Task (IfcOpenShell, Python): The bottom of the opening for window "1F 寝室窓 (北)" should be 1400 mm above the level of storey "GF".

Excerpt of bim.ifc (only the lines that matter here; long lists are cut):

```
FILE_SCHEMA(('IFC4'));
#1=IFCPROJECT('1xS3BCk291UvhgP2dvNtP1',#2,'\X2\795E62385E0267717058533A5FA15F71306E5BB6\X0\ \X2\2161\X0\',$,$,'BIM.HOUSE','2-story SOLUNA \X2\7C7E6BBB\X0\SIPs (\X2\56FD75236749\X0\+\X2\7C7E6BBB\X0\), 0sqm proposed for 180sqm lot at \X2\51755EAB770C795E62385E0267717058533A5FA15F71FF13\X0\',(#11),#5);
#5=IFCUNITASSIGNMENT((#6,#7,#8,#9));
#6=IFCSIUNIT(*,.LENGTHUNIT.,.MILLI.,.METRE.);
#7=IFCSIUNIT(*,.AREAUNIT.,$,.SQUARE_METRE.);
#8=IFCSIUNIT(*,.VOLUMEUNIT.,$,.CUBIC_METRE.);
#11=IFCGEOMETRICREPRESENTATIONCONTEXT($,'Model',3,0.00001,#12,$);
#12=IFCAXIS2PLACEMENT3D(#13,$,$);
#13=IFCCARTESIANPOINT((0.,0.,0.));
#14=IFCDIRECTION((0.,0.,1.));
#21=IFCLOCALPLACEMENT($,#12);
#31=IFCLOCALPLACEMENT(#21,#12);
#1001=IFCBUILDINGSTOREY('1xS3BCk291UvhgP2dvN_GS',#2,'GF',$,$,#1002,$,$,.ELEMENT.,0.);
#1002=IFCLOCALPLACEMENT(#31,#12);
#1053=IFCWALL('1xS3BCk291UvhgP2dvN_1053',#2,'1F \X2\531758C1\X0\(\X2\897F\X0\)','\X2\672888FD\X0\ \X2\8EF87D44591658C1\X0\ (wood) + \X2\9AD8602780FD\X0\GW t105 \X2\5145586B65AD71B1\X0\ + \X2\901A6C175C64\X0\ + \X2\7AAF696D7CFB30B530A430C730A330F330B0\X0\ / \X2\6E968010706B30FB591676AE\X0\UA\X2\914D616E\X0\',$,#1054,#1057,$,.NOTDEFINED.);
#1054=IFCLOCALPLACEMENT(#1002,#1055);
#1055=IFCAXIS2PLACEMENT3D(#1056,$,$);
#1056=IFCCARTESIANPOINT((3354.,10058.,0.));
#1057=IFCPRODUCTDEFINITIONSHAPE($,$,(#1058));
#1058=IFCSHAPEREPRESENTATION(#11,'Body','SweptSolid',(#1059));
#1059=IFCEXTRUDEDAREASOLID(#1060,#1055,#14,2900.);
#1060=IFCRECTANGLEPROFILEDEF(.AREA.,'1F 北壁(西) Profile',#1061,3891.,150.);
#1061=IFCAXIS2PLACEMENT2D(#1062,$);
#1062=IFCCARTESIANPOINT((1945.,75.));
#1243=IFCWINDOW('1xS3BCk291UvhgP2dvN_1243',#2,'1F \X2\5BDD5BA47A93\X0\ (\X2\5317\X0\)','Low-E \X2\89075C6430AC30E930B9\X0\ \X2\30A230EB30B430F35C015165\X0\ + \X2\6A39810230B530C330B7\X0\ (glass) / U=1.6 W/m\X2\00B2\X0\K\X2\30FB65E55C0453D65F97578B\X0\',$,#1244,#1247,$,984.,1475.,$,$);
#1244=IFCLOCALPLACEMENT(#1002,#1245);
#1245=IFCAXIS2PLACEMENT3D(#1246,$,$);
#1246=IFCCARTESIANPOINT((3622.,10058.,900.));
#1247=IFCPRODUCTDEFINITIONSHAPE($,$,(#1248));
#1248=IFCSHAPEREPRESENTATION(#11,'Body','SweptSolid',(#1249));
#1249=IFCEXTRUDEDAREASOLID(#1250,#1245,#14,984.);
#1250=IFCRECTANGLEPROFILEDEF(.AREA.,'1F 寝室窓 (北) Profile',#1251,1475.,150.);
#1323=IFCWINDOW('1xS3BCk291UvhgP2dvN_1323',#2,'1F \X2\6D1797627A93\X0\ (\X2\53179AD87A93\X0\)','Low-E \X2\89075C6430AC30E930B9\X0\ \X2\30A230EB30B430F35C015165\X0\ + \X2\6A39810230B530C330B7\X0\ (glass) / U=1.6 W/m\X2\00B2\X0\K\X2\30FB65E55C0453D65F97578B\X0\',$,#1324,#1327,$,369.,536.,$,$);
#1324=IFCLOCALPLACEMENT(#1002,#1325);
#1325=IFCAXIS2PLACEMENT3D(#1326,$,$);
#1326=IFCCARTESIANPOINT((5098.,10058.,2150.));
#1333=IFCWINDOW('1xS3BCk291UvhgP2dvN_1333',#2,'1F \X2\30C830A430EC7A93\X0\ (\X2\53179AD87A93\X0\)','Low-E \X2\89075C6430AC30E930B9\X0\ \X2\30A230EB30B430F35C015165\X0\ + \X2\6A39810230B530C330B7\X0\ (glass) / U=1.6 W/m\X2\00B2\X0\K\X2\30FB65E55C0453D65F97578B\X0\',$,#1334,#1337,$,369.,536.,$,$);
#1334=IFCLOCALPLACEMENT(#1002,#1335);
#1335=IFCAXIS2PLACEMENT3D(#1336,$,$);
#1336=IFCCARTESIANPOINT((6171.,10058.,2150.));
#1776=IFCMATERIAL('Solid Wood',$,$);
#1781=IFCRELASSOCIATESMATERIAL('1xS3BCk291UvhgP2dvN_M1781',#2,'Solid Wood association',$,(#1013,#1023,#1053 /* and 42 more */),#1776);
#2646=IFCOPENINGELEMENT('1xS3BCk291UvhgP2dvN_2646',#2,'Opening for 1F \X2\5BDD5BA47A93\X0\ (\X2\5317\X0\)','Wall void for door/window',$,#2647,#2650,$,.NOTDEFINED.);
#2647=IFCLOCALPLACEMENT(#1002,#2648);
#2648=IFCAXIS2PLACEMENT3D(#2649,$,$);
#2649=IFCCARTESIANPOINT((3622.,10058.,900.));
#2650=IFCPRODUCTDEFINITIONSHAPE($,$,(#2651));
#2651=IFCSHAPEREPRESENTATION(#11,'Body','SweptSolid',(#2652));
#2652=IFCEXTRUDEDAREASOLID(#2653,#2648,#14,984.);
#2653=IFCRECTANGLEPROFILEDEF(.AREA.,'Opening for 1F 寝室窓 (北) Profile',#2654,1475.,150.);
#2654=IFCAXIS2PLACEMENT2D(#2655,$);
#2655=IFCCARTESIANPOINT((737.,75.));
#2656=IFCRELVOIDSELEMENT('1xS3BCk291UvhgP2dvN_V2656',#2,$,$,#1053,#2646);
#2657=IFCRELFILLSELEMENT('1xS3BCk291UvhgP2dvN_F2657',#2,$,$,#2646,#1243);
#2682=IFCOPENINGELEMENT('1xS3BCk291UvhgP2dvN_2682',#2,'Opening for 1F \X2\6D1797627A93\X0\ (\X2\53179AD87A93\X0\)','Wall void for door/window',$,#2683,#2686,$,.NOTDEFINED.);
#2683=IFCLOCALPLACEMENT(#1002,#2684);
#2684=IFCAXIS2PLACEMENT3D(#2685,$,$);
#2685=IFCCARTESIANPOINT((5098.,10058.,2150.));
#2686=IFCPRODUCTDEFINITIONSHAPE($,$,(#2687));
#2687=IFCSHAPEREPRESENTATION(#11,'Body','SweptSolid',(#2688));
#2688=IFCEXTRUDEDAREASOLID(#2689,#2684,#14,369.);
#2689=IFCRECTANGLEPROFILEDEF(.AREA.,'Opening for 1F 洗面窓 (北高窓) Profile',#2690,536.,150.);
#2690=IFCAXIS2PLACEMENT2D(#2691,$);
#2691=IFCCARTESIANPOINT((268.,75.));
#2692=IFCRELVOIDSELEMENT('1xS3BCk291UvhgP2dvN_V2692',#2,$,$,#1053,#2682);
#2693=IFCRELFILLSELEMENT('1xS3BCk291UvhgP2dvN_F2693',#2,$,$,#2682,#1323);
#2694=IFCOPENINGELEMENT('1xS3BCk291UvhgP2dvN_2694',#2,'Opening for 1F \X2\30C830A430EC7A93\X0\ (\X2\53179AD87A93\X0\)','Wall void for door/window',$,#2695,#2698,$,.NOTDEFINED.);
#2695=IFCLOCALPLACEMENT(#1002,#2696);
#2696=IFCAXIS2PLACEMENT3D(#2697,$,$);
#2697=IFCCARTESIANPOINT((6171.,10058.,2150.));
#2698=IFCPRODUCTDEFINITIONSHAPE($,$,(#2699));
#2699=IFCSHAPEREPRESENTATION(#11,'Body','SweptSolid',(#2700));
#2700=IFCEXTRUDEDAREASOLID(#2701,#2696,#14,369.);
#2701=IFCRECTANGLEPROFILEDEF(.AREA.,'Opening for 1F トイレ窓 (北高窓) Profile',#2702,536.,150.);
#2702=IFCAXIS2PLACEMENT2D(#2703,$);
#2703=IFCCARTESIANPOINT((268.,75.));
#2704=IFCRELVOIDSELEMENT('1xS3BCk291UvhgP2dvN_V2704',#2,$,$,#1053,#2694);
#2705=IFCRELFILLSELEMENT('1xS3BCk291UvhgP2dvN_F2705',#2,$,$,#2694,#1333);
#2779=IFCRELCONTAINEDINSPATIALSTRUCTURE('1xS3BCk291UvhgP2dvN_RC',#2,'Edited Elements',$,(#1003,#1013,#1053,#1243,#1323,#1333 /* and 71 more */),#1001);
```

```python
import numpy as np
import ifcopenshell
import ifcopenshell.api.geometry
import ifcopenshell.geom
import ifcopenshell.util.element
import ifcopenshell.util.placement
import ifcopenshell.util.shape
import ifcopenshell.util.unit

model = ifcopenshell.open("bim.ifc")
unit_scale = ifcopenshell.util.unit.calculate_unit_scale(model)

window = model.by_guid("1xS3BCk291UvhgP2dvN_1243")
opening = window.FillsVoids[0].RelatingOpeningElement
storey = ifcopenshell.util.element.get_container(window, ifc_class="IfcBuildingStorey")
level = ifcopenshell.util.placement.get_local_placement(storey.ObjectPlacement)[2, 3]

# The opening's origin need not be at the sill, so measure its lowest point.
shape = ifcopenshell.geom.create_shape(ifcopenshell.geom.settings(), opening)
bottom = ifcopenshell.util.shape.get_shape_bottom_elevation(shape, shape.geometry) / unit_scale
dz = level + 1400.0 - bottom

shift = np.array([0.0, 0.0, dz])
# The window is not placed relative to its opening, so move both.
for product in (opening, window):
    matrix = ifcopenshell.util.placement.get_local_placement(product.ObjectPlacement)
    matrix[:3, 3] += shift
    ifcopenshell.api.geometry.edit_object_placement(model, product=product, matrix=matrix, is_si=False)

print(f"moved by {dz * unit_scale:+.3f} m")

model.write("bim_edited.ifc")
```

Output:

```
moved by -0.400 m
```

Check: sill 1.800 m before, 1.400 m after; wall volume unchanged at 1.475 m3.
